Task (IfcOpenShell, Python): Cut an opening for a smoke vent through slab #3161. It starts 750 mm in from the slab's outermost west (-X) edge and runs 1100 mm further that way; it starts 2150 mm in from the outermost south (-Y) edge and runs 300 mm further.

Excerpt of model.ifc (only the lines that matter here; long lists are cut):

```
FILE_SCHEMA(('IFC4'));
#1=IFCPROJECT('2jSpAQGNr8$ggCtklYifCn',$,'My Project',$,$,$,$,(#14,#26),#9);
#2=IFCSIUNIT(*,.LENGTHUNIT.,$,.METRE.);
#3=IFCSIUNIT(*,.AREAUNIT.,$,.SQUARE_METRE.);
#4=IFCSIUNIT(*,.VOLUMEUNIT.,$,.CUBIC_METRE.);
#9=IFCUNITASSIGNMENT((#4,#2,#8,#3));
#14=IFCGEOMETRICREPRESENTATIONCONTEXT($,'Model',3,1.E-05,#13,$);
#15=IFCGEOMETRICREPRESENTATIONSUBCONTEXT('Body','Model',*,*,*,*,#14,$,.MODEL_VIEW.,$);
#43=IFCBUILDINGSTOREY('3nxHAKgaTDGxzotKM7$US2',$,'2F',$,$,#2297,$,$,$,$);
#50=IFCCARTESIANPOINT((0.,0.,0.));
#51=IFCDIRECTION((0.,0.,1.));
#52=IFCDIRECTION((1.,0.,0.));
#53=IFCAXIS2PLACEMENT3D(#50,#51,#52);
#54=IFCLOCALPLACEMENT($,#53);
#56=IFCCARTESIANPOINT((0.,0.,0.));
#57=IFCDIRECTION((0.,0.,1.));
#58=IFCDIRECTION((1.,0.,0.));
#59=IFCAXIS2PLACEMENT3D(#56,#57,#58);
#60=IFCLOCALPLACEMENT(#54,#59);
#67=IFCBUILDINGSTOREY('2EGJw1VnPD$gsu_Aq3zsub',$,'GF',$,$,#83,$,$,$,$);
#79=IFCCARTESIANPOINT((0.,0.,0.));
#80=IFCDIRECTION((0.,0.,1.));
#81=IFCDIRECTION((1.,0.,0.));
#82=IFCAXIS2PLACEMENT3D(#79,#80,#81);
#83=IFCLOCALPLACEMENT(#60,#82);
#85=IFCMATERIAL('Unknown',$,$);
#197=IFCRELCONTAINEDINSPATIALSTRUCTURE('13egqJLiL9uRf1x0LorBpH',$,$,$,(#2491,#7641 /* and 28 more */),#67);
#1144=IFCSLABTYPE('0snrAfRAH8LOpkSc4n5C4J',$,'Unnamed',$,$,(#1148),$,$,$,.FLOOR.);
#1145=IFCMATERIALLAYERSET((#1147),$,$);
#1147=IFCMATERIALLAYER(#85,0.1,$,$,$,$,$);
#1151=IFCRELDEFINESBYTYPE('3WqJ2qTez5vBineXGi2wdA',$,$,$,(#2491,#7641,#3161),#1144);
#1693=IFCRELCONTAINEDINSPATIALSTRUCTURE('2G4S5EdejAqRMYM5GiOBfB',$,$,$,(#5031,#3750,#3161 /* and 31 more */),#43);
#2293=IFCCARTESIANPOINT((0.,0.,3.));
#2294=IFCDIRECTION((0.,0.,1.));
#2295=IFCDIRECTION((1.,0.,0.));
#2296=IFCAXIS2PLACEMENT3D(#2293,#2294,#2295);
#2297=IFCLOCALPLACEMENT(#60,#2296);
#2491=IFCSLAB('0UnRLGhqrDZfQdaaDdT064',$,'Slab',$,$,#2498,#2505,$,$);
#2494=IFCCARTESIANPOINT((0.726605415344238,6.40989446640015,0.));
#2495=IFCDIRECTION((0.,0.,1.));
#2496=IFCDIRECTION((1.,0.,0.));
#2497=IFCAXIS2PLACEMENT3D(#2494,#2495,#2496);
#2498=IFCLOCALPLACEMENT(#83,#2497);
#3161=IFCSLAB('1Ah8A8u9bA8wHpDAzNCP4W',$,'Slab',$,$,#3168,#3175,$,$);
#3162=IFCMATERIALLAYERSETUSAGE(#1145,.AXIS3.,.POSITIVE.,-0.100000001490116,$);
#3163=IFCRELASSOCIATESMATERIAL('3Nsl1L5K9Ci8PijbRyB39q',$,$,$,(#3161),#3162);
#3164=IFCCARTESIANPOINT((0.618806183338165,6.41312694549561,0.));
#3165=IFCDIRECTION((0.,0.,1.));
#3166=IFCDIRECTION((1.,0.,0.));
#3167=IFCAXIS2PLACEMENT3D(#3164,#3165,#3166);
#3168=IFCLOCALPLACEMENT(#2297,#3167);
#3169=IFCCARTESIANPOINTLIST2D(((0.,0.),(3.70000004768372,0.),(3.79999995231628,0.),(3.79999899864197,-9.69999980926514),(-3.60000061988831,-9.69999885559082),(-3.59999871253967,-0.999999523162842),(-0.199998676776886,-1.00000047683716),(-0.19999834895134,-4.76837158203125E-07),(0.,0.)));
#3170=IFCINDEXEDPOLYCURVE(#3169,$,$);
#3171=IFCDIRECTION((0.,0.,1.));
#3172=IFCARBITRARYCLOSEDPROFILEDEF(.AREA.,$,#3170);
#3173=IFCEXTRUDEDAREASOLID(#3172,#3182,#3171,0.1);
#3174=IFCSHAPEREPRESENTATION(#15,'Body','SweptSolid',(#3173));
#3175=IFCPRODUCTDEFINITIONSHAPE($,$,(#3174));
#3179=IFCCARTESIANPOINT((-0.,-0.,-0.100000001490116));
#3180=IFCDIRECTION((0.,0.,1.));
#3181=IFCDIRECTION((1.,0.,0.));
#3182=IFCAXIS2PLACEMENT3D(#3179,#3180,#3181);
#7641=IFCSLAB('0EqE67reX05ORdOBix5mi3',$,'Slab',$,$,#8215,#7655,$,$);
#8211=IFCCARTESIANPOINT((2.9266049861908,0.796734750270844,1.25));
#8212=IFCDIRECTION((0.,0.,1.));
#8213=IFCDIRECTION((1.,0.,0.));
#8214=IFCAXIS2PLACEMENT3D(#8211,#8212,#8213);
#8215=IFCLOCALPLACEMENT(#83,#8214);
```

```python
import numpy as np
import ifcopenshell
import ifcopenshell.api.feature
import ifcopenshell.api.geometry
import ifcopenshell.api.root
import ifcopenshell.geom
import ifcopenshell.util.placement
import ifcopenshell.util.representation
import ifcopenshell.util.shape
import ifcopenshell.util.unit

model = ifcopenshell.open("model.ifc")
unit_scale = ifcopenshell.util.unit.calculate_unit_scale(model)
settings = ifcopenshell.geom.settings()


def volume(element):
    """Net volume in cubic metres, openings subtracted."""
    shape = ifcopenshell.geom.create_shape(settings, element)
    return ifcopenshell.util.shape.get_volume(shape.geometry)


slab = model.by_id(3161)
before = volume(slab)

# Extent in the slab's own axes, in metres. The edges named are its -X and -Y sides.
slab_shape = ifcopenshell.geom.create_shape(settings, slab)
vertices = ifcopenshell.util.shape.get_vertices(slab_shape.geometry)
x_min, y_min, bottom = vertices.min(axis=0)
top = vertices[:, 2].max()

opening = ifcopenshell.api.root.create_entity(model, ifc_class="IfcOpeningElement", name="Smoke vent opening", predefined_type="OPENING")
context = ifcopenshell.util.representation.get_context(model, "Model", "Body", "MODEL_VIEW")
width, depth = 1.1, 0.3
outline = [(0.0, 0.0), (width, 0.0), (width, depth), (0.0, depth), (0.0, 0.0)]
# Overshoot both faces by 50 mm so the cut is clean.
shape = ifcopenshell.api.geometry.add_slab_representation(
    model, context=context, depth=top - bottom + 0.1, polyline=outline
)
ifcopenshell.api.geometry.assign_representation(model, product=opening, representation=shape)

matrix = ifcopenshell.util.placement.get_local_placement(slab.ObjectPlacement)
matrix[:, 3] = matrix @ np.append(np.array([x_min + 0.75, y_min + 2.15, bottom - 0.05]) / unit_scale, 1.0)
ifcopenshell.api.geometry.edit_object_placement(model, product=opening, matrix=matrix, is_si=False)
ifcopenshell.api.feature.add_feature(model, feature=opening, element=slab)

after = volume(slab)

print(f"slab volume {before:.3f} -> {after:.3f} m3")

model.write("model_rev.ifc")
```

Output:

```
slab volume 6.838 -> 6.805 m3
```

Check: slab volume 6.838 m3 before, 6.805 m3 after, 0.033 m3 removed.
